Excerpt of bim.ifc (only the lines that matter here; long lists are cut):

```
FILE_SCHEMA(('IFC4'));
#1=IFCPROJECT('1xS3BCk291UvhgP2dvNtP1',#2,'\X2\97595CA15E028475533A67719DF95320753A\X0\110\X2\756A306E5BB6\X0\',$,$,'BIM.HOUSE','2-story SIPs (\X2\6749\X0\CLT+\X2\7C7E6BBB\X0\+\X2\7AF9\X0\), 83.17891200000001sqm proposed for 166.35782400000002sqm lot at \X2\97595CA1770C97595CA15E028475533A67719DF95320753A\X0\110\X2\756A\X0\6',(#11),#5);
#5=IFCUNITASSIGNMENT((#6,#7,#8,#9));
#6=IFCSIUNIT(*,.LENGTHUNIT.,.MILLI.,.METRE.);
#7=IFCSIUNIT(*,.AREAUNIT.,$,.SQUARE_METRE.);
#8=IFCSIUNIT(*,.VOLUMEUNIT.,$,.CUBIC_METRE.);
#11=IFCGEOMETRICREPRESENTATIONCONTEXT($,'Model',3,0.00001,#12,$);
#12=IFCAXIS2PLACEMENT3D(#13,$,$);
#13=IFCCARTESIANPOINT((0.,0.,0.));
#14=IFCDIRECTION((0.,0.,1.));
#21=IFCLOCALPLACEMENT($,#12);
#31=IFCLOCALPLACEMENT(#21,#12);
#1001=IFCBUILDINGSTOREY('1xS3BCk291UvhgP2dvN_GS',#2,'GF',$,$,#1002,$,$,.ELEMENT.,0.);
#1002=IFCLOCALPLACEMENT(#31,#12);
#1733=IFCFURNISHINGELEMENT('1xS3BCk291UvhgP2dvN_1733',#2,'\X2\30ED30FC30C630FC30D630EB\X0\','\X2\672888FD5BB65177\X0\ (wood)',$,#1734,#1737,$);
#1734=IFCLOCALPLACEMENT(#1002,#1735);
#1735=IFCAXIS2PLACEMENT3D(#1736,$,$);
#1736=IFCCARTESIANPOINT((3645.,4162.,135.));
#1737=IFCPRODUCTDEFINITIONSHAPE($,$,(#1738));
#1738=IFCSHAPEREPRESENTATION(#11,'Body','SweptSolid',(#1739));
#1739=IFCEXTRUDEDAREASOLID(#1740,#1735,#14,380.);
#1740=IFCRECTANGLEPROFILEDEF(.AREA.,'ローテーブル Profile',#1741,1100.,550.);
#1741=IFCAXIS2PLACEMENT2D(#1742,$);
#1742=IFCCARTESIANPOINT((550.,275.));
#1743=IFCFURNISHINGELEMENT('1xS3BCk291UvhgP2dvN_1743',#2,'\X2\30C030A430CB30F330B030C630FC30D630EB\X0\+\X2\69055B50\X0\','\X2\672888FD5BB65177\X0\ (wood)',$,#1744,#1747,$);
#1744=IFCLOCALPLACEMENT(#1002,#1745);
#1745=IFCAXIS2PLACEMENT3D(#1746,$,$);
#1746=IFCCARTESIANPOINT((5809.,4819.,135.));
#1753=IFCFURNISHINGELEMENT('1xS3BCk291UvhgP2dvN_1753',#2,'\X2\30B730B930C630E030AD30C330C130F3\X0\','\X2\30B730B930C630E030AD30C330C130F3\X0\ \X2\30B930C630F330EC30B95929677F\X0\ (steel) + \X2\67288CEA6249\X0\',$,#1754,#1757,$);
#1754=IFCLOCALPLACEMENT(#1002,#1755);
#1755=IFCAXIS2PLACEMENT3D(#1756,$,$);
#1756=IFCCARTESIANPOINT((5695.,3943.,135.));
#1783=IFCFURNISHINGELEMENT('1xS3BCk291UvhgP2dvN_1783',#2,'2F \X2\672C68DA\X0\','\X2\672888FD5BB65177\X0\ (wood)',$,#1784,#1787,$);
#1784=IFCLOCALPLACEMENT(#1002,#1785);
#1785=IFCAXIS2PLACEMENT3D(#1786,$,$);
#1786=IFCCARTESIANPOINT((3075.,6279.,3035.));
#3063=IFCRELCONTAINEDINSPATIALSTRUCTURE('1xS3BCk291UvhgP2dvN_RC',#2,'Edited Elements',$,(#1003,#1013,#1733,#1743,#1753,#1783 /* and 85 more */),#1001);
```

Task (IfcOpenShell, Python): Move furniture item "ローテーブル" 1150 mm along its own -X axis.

```python
import ifcopenshell
import ifcopenshell.api.geometry
import ifcopenshell.util.placement
import ifcopenshell.util.unit

model = ifcopenshell.open("bim.ifc")
unit_scale = ifcopenshell.util.unit.calculate_unit_scale(model)

item = model.by_guid("1xS3BCk291UvhgP2dvN_1733")
matrix = ifcopenshell.util.placement.get_local_placement(item.ObjectPlacement)
matrix[:3, 3] -= matrix[:3, 0] * 1.15 / unit_scale
ifcopenshell.api.geometry.edit_object_placement(model, product=item, matrix=matrix, is_si=False)

print(ifcopenshell.util.placement.get_local_placement(item.ObjectPlacement).round(3) + 0.0)

model.write("bim_v2.ifc")
```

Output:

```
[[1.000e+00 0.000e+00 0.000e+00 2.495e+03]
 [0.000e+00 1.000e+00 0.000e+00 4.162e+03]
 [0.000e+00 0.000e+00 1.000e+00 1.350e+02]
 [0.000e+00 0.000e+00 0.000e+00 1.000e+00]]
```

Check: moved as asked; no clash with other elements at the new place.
